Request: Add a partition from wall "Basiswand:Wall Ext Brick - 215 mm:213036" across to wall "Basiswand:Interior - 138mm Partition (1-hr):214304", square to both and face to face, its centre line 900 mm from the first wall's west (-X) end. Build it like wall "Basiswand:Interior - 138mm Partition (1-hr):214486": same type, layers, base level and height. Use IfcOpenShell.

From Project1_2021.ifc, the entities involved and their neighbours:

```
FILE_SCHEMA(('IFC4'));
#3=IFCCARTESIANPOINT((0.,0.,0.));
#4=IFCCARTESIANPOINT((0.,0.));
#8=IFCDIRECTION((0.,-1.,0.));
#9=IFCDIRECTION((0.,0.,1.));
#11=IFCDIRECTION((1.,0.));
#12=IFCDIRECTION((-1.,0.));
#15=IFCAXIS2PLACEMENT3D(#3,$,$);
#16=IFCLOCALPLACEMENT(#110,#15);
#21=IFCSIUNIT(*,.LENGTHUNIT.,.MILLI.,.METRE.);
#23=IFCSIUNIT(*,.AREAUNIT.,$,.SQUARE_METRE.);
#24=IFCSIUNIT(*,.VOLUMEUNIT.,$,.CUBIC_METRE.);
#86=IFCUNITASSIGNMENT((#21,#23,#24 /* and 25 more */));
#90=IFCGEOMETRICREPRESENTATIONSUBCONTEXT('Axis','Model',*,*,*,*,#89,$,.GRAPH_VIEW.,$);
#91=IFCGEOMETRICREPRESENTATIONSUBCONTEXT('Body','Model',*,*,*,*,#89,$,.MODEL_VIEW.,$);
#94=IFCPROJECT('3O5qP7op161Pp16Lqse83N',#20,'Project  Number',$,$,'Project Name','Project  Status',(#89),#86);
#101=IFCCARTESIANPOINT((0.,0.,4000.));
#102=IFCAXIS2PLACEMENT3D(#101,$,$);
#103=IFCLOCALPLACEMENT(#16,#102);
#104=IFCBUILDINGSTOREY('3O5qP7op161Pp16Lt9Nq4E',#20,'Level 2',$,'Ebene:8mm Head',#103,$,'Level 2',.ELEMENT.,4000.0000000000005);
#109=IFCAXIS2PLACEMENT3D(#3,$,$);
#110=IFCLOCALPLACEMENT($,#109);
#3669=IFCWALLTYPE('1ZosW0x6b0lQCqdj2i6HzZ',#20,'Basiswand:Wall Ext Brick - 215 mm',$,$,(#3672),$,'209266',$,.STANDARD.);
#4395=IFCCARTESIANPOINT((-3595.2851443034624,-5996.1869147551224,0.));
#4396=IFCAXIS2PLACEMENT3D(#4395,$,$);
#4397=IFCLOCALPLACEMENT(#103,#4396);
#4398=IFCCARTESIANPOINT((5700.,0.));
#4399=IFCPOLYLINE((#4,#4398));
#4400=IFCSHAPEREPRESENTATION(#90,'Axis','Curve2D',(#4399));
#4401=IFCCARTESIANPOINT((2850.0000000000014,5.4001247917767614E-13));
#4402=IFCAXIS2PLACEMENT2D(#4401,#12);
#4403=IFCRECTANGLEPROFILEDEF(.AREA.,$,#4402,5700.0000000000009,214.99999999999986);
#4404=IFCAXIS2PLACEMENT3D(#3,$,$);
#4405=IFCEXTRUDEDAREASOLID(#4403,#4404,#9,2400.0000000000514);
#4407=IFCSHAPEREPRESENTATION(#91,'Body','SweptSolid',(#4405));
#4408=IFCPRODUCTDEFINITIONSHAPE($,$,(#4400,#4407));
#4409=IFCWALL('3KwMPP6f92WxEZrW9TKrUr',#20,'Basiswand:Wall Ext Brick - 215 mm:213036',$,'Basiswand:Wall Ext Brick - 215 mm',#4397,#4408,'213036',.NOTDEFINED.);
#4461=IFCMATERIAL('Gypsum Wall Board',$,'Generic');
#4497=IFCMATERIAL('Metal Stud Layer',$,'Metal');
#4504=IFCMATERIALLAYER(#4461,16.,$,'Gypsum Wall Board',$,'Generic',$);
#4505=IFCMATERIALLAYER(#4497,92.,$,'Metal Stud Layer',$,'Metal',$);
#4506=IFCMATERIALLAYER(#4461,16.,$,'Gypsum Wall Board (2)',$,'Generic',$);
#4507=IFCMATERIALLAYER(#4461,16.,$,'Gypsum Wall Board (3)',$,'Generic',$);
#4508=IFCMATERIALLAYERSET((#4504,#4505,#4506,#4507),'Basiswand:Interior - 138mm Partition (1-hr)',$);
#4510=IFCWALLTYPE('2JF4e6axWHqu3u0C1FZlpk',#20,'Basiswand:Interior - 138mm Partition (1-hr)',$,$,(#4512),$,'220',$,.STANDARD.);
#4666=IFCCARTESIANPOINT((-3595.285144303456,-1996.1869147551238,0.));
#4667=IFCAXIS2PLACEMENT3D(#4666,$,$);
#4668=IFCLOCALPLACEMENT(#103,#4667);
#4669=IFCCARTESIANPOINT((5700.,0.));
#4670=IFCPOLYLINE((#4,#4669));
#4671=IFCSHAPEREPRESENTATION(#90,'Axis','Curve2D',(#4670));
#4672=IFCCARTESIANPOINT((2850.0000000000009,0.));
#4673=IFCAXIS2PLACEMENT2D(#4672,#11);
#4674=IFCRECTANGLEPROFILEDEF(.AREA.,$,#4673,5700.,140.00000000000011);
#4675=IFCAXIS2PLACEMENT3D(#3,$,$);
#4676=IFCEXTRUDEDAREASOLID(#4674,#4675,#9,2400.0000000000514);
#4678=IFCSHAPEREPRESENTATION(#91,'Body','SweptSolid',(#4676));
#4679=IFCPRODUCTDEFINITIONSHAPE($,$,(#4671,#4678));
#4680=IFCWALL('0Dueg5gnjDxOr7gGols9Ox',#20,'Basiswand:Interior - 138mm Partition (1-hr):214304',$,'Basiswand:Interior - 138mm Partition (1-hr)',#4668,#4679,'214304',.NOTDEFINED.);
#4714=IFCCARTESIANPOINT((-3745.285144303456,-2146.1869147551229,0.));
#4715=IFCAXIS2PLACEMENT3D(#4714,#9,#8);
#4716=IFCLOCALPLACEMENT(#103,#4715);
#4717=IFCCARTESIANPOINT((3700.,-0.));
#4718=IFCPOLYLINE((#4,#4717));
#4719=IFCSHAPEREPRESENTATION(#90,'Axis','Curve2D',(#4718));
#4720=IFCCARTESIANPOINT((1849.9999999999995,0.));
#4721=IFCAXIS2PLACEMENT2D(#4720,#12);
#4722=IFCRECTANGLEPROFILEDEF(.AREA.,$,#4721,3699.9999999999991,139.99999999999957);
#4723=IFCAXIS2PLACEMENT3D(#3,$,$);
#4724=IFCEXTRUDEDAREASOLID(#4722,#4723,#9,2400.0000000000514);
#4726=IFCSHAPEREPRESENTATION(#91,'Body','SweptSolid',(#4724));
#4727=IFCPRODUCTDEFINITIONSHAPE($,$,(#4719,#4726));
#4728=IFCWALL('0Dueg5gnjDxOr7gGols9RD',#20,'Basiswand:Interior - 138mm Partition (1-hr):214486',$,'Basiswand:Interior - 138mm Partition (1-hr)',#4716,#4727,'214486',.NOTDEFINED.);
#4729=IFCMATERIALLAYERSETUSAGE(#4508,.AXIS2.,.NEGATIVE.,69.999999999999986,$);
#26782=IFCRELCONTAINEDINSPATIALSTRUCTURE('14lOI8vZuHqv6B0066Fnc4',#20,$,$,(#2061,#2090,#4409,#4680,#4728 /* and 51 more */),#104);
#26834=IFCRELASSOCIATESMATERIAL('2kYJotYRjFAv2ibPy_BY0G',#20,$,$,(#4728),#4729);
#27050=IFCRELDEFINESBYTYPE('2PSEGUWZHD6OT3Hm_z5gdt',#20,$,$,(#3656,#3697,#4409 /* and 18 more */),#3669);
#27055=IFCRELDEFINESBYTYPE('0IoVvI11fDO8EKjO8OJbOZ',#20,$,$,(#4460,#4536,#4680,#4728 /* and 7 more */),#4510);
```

```python
import numpy as np
import ifcopenshell
import ifcopenshell.api.geometry
import ifcopenshell.api.material
import ifcopenshell.api.pset
import ifcopenshell.api.root
import ifcopenshell.api.spatial
import ifcopenshell.api.type
import ifcopenshell.geom
import ifcopenshell.util.element
import ifcopenshell.util.placement
import ifcopenshell.util.representation
import ifcopenshell.util.shape
import ifcopenshell.util.unit

model = ifcopenshell.open("Project1_2021.ifc")
unit_scale = ifcopenshell.util.unit.calculate_unit_scale(model)
settings = ifcopenshell.geom.settings()
settings.set("use-world-coords", True)

start_wall = model.by_guid("3KwMPP6f92WxEZrW9TKrUr")
end_wall = model.by_guid("0Dueg5gnjDxOr7gGols9Ox")
like = model.by_id(4728)
matrix = ifcopenshell.util.placement.get_local_placement(start_wall.ObjectPlacement)
matrix[:3, 3] *= unit_scale


def extent(element):
    """Bounding box in the first wall's axes, in metres."""
    shape = ifcopenshell.geom.create_shape(settings, element)
    points = (ifcopenshell.util.shape.get_vertices(shape.geometry) - matrix[:3, 3]) @ matrix[:3, :3]
    return points.min(axis=0), points.max(axis=0)


y_start = extent(start_wall)[1][1]
y_end = extent(end_wall)[0][1]
like_min, like_max = extent(like)
length, height = float(abs(y_end - y_start)), float(like_max[2] - like_min[2])
layer_set = ifcopenshell.util.element.get_material(like, should_skip_usage=True)
thickness = sum(layer.LayerThickness for layer in layer_set.MaterialLayers) * unit_scale

wall = ifcopenshell.api.root.create_entity(model, ifc_class="IfcWall", name="New partition")
storey = ifcopenshell.util.element.get_container(like)
ifcopenshell.api.spatial.assign_container(model, products=[wall], relating_structure=storey)
ifcopenshell.api.type.assign_type(
    model, related_objects=[wall], relating_type=ifcopenshell.util.element.get_type(like), should_map_representations=False
)
rel = ifcopenshell.api.material.assign_material(
    model, products=[wall], type="IfcMaterialLayerSetUsage", material=layer_set
)
rel.RelatingMaterial.OffsetFromReferenceLine = -thickness / 2 / unit_scale
pset = ifcopenshell.api.pset.add_pset(model, product=wall, name="Pset_WallCommon")
ifcopenshell.api.pset.edit_pset(model, pset=pset, properties={"IsExternal": False, "LoadBearing": False})

# The axis runs down the middle of the wall.
axis = ifcopenshell.api.geometry.add_axis_representation(
    model, context=ifcopenshell.util.representation.get_context(model, "Model", "Axis"), axis=[(0.0, 0.0), (length, 0.0)]
)
body = ifcopenshell.api.geometry.add_wall_representation(
    model,
    context=ifcopenshell.util.representation.get_context(model, "Model", "Body", "MODEL_VIEW"),
    length=length,
    height=height,
    thickness=thickness,
    offset=-thickness / 2,
)
for representation in (axis, body):
    ifcopenshell.api.geometry.assign_representation(model, product=wall, representation=representation)

placement = matrix @ ifcopenshell.util.placement.rotation(90, "Z")
placement[:, 3] = matrix @ np.array([extent(start_wall)[0][0] + 0.9, y_start, like_min[2], 1.0])
ifcopenshell.api.geometry.edit_object_placement(model, product=wall, matrix=placement)

print(f"partition {length:.3f} m long, {height:.3f} m high, {thickness:.3f} m thick")

model.write("Project1_2021_v2.ifc")
```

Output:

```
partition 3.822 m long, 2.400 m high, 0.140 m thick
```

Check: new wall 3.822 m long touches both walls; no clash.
